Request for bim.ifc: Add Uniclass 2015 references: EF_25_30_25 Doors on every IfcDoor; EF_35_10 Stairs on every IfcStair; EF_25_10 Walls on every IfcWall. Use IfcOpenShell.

First a look at what the model holds.

```python
import ifcopenshell

model = ifcopenshell.open("bim.ifc")
print(model.schema)
print("classifications:", [c.Name for c in model.by_type("IfcClassification")])
for ifc_class in ("IfcDoor", "IfcRoof", "IfcStair", "IfcWall", "IfcWindow"):
    print(ifc_class, len(model.by_type(ifc_class)))
```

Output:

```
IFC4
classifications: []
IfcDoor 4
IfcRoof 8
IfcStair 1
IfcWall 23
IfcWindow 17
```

```python
import ifcopenshell
import ifcopenshell.api.classification

model = ifcopenshell.open("bim.ifc")

system = ifcopenshell.api.classification.add_classification(model, classification="Uniclass 2015")

codes = {
    "IfcDoor": ("EF_25_30_25", "Doors"),
    "IfcStair": ("EF_35_10", "Stairs"),
    "IfcWall": ("EF_25_10", "Walls"),
}
for ifc_class, (code, name) in codes.items():
    products = model.by_type(ifc_class)
    ifcopenshell.api.classification.add_reference(
        model, products=products, classification=system, identification=code, name=name
    )
    print(code, len(products))

model.write("bim_rev.ifc")
```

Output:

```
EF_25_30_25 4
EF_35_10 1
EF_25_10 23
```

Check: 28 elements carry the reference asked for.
